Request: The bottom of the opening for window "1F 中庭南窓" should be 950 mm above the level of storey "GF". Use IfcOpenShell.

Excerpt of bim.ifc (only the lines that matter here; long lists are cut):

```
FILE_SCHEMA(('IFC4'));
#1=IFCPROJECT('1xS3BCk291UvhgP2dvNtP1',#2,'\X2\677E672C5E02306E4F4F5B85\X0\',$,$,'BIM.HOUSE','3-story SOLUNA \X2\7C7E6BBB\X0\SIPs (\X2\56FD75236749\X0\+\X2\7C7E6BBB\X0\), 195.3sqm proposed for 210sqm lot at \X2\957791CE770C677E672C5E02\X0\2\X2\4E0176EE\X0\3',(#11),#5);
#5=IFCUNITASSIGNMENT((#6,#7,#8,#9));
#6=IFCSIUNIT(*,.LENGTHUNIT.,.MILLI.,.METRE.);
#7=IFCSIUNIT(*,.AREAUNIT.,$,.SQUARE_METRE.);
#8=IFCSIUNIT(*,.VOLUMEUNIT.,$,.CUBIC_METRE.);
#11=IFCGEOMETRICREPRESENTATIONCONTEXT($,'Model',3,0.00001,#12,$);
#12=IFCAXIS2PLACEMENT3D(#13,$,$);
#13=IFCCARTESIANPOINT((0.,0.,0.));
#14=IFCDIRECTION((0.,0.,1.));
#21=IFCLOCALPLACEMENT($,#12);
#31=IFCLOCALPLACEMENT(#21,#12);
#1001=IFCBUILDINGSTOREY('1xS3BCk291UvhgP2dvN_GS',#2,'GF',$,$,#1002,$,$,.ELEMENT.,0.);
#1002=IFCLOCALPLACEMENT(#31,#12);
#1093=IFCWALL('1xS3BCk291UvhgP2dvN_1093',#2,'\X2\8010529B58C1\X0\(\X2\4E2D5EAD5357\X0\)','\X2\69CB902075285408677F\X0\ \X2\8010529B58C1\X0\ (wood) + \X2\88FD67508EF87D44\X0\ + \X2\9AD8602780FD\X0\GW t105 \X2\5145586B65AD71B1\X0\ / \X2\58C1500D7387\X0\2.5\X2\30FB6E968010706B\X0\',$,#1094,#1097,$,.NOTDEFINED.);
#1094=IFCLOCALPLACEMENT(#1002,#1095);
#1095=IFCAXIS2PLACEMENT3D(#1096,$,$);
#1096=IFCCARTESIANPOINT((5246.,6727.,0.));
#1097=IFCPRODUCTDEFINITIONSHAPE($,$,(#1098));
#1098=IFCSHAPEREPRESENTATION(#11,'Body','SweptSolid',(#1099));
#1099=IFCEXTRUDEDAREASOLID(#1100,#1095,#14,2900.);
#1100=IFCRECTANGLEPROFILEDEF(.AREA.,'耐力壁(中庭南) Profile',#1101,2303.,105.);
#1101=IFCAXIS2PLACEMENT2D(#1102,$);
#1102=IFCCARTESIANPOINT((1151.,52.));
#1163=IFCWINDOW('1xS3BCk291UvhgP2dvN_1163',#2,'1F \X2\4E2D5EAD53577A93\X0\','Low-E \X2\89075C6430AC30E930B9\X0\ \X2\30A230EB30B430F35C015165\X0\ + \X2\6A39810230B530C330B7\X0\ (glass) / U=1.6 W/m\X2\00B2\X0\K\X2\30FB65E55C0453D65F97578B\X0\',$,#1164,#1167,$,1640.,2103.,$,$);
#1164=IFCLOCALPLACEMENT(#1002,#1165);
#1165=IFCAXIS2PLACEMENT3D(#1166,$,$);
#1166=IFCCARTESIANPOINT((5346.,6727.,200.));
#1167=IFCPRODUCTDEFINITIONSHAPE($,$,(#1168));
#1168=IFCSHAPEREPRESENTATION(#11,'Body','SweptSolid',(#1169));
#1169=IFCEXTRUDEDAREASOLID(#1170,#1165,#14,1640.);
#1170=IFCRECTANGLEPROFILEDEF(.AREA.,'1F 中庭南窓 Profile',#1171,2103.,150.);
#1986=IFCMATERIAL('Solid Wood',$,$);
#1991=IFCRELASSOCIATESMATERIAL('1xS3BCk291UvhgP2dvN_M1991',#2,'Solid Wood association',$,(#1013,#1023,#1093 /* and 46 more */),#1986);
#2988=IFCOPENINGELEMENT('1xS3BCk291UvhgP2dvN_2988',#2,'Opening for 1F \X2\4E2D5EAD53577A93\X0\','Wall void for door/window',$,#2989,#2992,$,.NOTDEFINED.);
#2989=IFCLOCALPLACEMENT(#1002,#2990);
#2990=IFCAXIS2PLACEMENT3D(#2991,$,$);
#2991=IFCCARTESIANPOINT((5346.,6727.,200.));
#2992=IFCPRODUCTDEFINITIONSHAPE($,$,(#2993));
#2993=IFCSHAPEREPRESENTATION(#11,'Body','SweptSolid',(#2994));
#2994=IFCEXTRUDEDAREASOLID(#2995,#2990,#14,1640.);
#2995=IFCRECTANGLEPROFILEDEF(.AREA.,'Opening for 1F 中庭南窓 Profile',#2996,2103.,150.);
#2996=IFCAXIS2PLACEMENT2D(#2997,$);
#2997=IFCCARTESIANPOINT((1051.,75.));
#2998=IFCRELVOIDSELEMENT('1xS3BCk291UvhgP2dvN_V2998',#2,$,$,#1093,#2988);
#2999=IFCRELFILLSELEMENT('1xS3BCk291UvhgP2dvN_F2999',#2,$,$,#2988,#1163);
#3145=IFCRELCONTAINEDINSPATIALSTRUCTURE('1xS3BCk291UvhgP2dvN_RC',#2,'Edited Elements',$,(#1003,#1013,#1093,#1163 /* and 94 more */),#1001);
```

```python
import numpy as np
import ifcopenshell
import ifcopenshell.api.geometry
import ifcopenshell.geom
import ifcopenshell.util.element
import ifcopenshell.util.placement
import ifcopenshell.util.shape
import ifcopenshell.util.unit

model = ifcopenshell.open("bim.ifc")
unit_scale = ifcopenshell.util.unit.calculate_unit_scale(model)

window = model.by_guid("1xS3BCk291UvhgP2dvN_1163")
opening = window.FillsVoids[0].RelatingOpeningElement
storey = ifcopenshell.util.element.get_container(window, ifc_class="IfcBuildingStorey")
level = ifcopenshell.util.placement.get_local_placement(storey.ObjectPlacement)[2, 3]

# The opening's origin need not be at the sill, so measure its lowest point.
shape = ifcopenshell.geom.create_shape(ifcopenshell.geom.settings(), opening)
bottom = ifcopenshell.util.shape.get_shape_bottom_elevation(shape, shape.geometry) / unit_scale
dz = level + 0.95 / unit_scale - bottom

shift = np.array([0.0, 0.0, dz])
# The window is not placed relative to its opening, so move both.
for product in (opening, window):
    matrix = ifcopenshell.util.placement.get_local_placement(product.ObjectPlacement)
    matrix[:3, 3] += shift
    ifcopenshell.api.geometry.edit_object_placement(model, product=product, matrix=matrix, is_si=False)

print(f"moved by {dz * unit_scale:+.3f} m")

model.write("bim_edited.ifc")
```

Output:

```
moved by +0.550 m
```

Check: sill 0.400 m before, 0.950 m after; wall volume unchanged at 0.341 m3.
